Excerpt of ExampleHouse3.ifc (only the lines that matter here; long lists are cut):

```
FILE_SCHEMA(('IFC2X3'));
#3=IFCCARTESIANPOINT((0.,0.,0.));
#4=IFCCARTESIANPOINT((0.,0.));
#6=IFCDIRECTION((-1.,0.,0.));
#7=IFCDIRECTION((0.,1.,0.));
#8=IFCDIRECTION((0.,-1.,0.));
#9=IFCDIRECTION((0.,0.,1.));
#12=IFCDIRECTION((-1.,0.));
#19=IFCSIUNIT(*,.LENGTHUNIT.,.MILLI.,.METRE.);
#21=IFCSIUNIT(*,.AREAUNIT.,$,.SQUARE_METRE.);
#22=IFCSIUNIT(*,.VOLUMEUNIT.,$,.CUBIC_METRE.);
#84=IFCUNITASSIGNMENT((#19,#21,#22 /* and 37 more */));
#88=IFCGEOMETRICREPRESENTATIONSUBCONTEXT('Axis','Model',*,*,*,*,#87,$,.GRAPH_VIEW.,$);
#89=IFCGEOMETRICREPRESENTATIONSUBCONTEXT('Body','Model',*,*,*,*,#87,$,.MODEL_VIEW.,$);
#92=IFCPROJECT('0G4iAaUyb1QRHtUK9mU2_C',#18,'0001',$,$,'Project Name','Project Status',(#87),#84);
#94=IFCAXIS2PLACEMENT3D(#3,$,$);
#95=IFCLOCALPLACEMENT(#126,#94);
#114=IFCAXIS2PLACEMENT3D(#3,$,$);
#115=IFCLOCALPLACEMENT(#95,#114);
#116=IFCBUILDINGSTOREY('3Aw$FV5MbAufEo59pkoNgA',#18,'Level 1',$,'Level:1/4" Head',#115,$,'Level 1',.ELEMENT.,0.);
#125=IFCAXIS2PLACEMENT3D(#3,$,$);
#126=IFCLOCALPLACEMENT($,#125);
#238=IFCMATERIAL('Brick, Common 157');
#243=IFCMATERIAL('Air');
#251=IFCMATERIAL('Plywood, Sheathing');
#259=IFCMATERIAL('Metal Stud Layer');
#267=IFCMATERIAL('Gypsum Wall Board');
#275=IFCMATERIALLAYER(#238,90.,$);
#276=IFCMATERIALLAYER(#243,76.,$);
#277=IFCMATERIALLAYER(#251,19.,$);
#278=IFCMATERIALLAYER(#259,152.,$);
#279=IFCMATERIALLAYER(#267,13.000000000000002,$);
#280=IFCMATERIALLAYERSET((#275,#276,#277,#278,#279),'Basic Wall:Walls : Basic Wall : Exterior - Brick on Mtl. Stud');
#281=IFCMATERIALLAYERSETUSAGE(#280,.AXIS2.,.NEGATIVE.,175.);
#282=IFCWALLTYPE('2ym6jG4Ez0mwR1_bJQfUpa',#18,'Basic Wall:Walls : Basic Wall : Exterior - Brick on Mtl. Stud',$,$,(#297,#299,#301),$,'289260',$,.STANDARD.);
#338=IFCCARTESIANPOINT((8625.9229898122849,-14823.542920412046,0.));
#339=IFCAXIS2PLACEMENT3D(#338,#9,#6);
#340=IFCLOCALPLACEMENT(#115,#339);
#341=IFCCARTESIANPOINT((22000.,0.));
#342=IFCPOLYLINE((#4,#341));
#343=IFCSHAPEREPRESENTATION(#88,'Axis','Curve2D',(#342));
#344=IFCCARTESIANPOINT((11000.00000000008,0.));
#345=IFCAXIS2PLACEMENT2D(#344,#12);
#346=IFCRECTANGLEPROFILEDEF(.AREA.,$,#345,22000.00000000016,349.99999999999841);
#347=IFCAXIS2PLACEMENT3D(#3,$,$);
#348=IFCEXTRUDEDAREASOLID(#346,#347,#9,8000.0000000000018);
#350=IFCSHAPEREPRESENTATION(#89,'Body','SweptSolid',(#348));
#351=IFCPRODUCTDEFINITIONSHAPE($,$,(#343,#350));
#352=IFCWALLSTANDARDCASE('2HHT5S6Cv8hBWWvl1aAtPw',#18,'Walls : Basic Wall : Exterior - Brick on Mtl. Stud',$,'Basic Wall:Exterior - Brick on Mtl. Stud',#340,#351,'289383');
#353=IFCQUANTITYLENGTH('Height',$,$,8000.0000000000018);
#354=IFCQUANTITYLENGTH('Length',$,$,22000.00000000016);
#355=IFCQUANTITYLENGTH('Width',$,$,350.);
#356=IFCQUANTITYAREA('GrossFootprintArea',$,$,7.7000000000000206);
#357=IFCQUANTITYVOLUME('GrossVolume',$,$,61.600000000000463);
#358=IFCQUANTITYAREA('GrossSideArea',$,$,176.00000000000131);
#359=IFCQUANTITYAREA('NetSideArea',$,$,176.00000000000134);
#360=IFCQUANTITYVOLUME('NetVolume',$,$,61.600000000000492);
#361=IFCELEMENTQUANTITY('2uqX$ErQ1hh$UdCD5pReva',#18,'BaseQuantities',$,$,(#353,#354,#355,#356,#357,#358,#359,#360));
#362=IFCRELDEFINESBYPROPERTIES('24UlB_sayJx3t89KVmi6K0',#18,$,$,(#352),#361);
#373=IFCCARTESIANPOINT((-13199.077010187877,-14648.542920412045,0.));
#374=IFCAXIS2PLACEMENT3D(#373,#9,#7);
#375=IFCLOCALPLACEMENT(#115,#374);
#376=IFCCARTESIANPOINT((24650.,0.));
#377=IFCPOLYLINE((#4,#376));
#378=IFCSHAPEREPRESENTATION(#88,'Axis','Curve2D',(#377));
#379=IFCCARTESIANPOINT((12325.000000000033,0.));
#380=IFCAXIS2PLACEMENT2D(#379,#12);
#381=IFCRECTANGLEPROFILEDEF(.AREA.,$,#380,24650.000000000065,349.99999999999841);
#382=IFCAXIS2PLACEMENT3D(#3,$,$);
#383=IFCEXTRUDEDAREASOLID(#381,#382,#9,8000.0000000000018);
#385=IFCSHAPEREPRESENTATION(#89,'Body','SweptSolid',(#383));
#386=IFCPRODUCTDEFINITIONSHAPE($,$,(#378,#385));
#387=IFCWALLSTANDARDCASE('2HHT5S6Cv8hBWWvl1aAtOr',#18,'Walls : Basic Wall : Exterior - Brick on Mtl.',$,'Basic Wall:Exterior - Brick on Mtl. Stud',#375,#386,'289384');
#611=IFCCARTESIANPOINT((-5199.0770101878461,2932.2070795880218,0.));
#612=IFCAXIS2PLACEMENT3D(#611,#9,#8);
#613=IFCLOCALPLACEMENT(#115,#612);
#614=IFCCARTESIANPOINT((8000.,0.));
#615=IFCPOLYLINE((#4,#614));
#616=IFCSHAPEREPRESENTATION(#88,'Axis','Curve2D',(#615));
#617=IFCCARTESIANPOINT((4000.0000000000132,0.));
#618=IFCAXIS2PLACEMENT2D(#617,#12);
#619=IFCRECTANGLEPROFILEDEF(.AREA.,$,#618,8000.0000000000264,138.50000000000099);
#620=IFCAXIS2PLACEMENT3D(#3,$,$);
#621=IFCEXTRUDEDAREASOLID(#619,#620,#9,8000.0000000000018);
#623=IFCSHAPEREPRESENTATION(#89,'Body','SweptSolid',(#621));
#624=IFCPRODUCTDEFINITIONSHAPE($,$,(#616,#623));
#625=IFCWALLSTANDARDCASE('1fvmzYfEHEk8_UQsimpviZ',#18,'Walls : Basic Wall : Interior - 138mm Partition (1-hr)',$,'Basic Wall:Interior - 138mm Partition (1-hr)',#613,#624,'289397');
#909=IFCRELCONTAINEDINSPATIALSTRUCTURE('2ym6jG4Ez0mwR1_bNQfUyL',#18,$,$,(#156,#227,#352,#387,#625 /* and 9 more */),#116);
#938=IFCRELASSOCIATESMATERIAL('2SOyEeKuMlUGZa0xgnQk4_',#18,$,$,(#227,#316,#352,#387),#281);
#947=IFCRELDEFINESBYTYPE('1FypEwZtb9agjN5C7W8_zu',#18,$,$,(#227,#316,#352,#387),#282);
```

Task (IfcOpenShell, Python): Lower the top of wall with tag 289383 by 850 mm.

```python
import ifcopenshell
import ifcopenshell.api.pset
import ifcopenshell.geom
import ifcopenshell.util.element
import ifcopenshell.util.representation
import ifcopenshell.util.shape
import ifcopenshell.util.unit

model = ifcopenshell.open("ExampleHouse3.ifc")
unit_scale = ifcopenshell.util.unit.calculate_unit_scale(model)
area_scale = ifcopenshell.util.unit.calculate_unit_scale(model, "AREAUNIT")
volume_scale = ifcopenshell.util.unit.calculate_unit_scale(model, "VOLUMEUNIT")
settings = ifcopenshell.geom.settings()


def volume(element):
    """Net volume in cubic metres, openings subtracted."""
    shape = ifcopenshell.geom.create_shape(settings, element)
    return ifcopenshell.util.shape.get_volume(shape.geometry)


wall = model.by_guid("2HHT5S6Cv8hBWWvl1aAtPw")
before = volume(wall)

body = ifcopenshell.util.representation.get_representation(wall, "Model", "Body")
solid = body.Items[0]
old_height = solid.Depth
solid.Depth -= 850.0
after = volume(wall)
thickness = 0.35  # wall thickness in metres

# Update the stored height, areas and volumes.
qto = model.by_id(ifcopenshell.util.element.get_pset(wall, "BaseQuantities", should_inherit=False)["id"])
ifcopenshell.api.pset.edit_qto(model, qto=qto, properties={
    "Height": solid.Depth,
    "GrossVolume": ifcopenshell.util.element.get_pset(wall, "BaseQuantities", "GrossVolume") * solid.Depth / old_height,
    "GrossSideArea": ifcopenshell.util.element.get_pset(wall, "BaseQuantities", "GrossSideArea") * solid.Depth / old_height,
    "NetSideArea": after / thickness / area_scale,
    "NetVolume": after / volume_scale,
})

print(f"height {old_height:g} -> {solid.Depth:g}, volume {before:.3f} -> {after:.3f} m3")

model.write("ExampleHouse3_rev.ifc")
```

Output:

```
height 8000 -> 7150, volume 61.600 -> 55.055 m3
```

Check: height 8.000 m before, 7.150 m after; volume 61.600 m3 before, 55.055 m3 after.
